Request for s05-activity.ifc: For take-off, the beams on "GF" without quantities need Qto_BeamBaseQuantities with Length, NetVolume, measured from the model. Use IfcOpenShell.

First a look at what the model holds.

```python
import ifcopenshell
import ifcopenshell.util.element
import ifcopenshell.util.unit

model = ifcopenshell.open("s05-activity.ifc")
print(model.schema)
for unit_type in ("LENGTHUNIT", "AREAUNIT", "VOLUMEUNIT"):
    print(unit_type, ifcopenshell.util.unit.calculate_unit_scale(model, unit_type))
storey = next(s for s in model.by_type("IfcBuildingStorey") if s.Name == "GF")
beams = [e for e in ifcopenshell.util.element.get_decomposition(storey) if e.is_a("IfcBeam")]
for e in sorted(beams, key=lambda e: e.id()):
    print(e.id(), e.is_a(), e.Name, list(ifcopenshell.util.element.get_psets(e, qtos_only=True)), sep=" | ")
```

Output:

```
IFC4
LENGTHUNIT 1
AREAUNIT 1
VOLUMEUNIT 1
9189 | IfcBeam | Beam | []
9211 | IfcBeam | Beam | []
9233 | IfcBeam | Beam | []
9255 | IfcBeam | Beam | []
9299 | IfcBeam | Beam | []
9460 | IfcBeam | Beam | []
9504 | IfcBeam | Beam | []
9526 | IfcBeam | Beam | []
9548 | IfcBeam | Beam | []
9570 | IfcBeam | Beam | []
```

```python
import ifcopenshell
import ifcopenshell.api.pset
import ifcopenshell.geom
import ifcopenshell.util.element
import ifcopenshell.util.shape
import ifcopenshell.util.unit

model = ifcopenshell.open("s05-activity.ifc")
unit_scale = ifcopenshell.util.unit.calculate_unit_scale(model)
volume_scale = ifcopenshell.util.unit.calculate_unit_scale(model, "VOLUMEUNIT")
settings = ifcopenshell.geom.settings()

storey = next(s for s in model.by_type("IfcBuildingStorey") if s.Name == "GF")
beams = [e for e in ifcopenshell.util.element.get_decomposition(storey) if e.is_a("IfcBeam")]

for e in sorted(beams, key=lambda e: e.id()):
    if ifcopenshell.util.element.get_psets(e, qtos_only=True, should_inherit=False):
        continue
    # Geometry comes back in metres, in the element's own axes.
    shape = ifcopenshell.geom.create_shape(settings, e)
    values = {
        "Length": ifcopenshell.util.shape.get_max_xyz(shape.geometry) / unit_scale,
        "NetVolume": ifcopenshell.util.shape.get_volume(shape.geometry) / volume_scale,
    }
    qto = ifcopenshell.api.pset.add_qto(model, product=e, name="Qto_BeamBaseQuantities")
    ifcopenshell.api.pset.edit_qto(model, qto=qto, properties=values)
    print(e.id(), {k: round(v, 3) for k, v in values.items()})

model.write("s05-activity_edited.ifc")
```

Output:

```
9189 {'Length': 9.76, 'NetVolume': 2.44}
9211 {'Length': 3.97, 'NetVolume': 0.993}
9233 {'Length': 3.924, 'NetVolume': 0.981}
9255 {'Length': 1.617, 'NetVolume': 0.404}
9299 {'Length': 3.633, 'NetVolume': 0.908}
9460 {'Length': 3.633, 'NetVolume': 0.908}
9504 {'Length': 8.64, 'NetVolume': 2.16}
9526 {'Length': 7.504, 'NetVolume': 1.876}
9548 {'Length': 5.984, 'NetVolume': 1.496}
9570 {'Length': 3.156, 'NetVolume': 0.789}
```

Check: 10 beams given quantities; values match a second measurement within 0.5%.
